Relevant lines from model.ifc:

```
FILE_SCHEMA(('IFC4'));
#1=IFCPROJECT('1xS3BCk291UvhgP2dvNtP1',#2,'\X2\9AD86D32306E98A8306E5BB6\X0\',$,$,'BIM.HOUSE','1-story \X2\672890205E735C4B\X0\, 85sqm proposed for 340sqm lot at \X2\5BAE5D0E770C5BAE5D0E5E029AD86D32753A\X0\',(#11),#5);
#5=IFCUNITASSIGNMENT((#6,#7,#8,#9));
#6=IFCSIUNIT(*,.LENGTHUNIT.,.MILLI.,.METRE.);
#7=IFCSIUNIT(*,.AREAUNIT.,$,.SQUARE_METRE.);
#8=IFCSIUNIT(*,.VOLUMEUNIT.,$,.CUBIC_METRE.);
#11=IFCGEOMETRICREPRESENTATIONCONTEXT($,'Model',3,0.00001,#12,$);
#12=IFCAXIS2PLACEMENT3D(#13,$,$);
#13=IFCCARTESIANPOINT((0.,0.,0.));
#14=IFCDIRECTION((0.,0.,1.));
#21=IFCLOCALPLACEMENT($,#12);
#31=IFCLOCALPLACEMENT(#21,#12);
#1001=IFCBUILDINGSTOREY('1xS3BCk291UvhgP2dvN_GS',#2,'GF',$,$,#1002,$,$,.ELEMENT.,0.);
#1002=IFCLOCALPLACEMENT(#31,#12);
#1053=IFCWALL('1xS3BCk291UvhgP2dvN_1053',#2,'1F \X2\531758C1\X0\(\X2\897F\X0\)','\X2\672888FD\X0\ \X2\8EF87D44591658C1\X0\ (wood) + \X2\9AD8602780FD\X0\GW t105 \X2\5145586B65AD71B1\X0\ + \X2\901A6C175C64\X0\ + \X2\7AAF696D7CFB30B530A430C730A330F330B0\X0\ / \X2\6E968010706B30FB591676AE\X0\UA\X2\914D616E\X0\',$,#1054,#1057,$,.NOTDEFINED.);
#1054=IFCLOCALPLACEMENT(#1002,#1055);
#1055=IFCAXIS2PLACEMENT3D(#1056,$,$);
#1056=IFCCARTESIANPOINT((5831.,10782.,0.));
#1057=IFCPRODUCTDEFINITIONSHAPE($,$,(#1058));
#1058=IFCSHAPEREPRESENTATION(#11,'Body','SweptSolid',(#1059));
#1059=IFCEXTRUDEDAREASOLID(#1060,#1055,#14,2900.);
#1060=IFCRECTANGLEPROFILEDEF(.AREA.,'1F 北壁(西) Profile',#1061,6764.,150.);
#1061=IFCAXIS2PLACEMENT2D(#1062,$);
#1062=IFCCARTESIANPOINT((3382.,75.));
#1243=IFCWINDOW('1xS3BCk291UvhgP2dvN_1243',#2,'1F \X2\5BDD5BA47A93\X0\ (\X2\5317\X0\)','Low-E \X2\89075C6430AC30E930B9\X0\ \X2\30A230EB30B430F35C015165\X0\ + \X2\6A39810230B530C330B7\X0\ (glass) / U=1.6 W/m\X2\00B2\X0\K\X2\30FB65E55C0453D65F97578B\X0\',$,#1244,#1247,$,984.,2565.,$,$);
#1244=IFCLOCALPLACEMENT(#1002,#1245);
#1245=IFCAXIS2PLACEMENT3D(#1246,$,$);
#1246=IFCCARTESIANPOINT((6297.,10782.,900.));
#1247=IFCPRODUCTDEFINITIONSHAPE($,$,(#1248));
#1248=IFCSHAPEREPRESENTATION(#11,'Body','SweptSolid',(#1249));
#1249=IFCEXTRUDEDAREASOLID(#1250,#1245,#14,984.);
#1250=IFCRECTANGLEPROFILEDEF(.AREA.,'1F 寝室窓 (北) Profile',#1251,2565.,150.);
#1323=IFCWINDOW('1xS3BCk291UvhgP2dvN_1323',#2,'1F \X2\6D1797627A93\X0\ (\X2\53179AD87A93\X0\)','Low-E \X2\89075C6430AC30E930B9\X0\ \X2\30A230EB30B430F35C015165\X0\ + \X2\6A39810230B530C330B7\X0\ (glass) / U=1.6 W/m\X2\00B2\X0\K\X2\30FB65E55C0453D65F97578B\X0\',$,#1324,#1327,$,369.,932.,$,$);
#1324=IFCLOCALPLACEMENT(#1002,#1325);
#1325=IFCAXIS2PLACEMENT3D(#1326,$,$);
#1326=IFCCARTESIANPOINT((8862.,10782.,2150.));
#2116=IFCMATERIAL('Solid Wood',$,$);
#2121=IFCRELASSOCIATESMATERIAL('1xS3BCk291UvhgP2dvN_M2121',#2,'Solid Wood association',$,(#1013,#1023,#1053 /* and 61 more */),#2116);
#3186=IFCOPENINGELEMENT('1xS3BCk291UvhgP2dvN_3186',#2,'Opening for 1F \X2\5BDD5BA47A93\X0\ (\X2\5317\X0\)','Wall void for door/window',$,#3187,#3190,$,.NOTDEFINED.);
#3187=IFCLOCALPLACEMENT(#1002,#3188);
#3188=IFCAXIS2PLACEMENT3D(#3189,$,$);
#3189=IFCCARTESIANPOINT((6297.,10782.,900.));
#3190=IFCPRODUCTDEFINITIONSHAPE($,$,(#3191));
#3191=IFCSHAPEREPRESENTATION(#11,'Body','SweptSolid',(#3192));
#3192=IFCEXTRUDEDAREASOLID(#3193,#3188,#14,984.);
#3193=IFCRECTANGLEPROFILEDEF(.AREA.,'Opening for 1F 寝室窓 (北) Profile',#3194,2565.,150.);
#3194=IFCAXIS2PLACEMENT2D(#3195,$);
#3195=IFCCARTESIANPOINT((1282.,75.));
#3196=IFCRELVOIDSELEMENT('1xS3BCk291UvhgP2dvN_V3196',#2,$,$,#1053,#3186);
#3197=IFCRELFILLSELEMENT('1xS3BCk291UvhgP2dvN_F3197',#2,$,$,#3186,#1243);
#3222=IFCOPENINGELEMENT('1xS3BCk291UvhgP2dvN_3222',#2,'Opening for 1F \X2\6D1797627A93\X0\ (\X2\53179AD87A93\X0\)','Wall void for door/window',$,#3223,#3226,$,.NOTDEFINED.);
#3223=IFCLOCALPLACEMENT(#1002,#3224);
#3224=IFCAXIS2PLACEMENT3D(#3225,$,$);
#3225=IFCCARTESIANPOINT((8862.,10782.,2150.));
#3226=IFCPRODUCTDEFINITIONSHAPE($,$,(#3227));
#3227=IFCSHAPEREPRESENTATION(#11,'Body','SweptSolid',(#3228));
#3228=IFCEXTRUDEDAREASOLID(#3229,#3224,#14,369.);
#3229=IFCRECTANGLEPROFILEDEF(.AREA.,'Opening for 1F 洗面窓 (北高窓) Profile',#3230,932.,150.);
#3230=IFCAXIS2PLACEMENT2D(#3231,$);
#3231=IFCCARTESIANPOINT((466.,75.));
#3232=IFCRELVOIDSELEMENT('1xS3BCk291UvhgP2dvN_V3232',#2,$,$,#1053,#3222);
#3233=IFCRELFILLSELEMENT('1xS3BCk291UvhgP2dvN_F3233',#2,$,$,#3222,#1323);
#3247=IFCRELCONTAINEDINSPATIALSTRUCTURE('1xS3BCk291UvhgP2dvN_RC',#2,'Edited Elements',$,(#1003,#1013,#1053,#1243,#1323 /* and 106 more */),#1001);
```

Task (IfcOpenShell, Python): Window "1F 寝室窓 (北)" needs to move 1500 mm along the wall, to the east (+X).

```python
import ifcopenshell
import ifcopenshell.api.geometry
import ifcopenshell.util.placement
import ifcopenshell.util.unit

model = ifcopenshell.open("model.ifc")
unit_scale = ifcopenshell.util.unit.calculate_unit_scale(model)

window = model.by_guid("1xS3BCk291UvhgP2dvN_1243")
opening = window.FillsVoids[0].RelatingOpeningElement
wall = opening.VoidsElements[0].RelatingBuildingElement

wall_matrix = ifcopenshell.util.placement.get_local_placement(wall.ObjectPlacement)
shift = wall_matrix[:3, 0] * 1.5 / unit_scale
before = ifcopenshell.util.placement.get_local_placement(window.ObjectPlacement)[:3, 3].copy()

# The window is not placed relative to its opening, so move both.
for product in (opening, window):
    matrix = ifcopenshell.util.placement.get_local_placement(product.ObjectPlacement)
    matrix[:3, 3] += shift
    ifcopenshell.api.geometry.edit_object_placement(model, product=product, matrix=matrix, is_si=False)

after = ifcopenshell.util.placement.get_local_placement(window.ObjectPlacement)[:3, 3]
print("window moved by", (after - before).round(3) + 0.0)

model.write("model-out.ifc")
```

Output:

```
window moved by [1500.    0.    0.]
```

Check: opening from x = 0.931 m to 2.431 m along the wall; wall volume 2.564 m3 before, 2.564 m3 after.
